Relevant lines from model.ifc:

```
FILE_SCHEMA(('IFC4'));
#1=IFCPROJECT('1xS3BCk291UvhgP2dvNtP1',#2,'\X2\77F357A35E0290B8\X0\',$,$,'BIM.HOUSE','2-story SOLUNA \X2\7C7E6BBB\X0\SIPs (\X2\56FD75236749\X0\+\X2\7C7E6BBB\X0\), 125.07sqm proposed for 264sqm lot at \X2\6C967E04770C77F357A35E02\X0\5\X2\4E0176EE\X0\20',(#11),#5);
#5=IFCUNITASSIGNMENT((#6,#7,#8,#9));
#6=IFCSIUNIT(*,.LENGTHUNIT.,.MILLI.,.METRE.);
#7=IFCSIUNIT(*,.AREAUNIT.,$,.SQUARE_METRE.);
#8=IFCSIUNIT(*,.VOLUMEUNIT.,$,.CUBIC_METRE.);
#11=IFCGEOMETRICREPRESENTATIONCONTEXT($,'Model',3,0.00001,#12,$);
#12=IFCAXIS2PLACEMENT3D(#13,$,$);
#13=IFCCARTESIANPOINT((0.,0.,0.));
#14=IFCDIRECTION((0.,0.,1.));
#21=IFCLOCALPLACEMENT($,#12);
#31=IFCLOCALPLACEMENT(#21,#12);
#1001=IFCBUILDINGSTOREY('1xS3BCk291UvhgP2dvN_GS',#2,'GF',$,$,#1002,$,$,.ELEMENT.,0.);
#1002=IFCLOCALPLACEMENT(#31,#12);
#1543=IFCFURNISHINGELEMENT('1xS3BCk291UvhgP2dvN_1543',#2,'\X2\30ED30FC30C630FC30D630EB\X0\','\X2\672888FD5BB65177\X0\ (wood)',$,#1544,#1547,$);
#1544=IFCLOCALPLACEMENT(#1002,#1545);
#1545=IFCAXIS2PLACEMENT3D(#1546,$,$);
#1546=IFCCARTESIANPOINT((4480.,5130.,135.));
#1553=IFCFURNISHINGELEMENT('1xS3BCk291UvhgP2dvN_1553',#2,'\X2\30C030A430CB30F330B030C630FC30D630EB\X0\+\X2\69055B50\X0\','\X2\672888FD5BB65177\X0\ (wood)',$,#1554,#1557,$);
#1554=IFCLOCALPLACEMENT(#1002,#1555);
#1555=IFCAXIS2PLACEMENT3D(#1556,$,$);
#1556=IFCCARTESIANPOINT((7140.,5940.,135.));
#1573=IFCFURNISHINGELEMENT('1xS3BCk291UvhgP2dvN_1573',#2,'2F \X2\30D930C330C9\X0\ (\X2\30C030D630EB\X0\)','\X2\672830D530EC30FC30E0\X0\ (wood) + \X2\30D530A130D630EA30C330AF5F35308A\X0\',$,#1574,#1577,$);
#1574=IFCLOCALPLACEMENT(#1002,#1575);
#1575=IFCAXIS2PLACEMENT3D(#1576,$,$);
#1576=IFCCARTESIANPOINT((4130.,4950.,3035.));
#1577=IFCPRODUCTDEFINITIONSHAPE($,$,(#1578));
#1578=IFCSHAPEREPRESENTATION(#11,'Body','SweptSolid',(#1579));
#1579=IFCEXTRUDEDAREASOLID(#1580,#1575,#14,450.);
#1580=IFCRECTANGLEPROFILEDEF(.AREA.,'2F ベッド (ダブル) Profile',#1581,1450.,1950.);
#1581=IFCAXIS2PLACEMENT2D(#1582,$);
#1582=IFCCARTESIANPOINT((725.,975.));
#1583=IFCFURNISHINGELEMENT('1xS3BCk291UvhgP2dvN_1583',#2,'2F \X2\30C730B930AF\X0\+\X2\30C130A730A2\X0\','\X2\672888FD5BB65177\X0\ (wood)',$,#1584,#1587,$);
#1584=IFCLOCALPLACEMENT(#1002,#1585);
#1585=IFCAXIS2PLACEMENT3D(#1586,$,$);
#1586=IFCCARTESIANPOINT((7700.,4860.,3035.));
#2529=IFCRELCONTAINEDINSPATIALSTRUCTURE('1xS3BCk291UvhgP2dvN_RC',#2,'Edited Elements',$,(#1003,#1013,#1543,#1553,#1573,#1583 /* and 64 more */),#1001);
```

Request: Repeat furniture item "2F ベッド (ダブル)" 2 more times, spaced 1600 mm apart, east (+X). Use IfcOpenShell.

```python
import numpy as np
import ifcopenshell
import ifcopenshell.api.geometry
import ifcopenshell.api.root
import ifcopenshell.util.element
import ifcopenshell.util.placement
import ifcopenshell.util.unit

model = ifcopenshell.open("model.ifc")
unit_scale = ifcopenshell.util.unit.calculate_unit_scale(model)


def reuse_history(source, copy):
    """copy_class also copies each property set's owner history, people and application; keep the originals."""
    for rel in copy.IsDefinedBy:
        if rel.is_a("IfcRelDefinesByProperties") and (history := rel.RelatingPropertyDefinition.OwnerHistory):
            rel.RelatingPropertyDefinition.OwnerHistory = source.OwnerHistory
            ifcopenshell.util.element.remove_deep2(model, history)


source = model.by_guid("1xS3BCk291UvhgP2dvN_1573")
base = ifcopenshell.util.placement.get_local_placement(source.ObjectPlacement)
step = np.array([1.0, 0.0, 0.0]) * 1.6 / unit_scale

for i in range(1, 3):
    copy = ifcopenshell.api.root.copy_class(model, product=source)
    copy.Representation = ifcopenshell.util.element.copy_deep(
        model, source.Representation, exclude=["IfcGeometricRepresentationContext", "IfcRepresentationMap"]
    )
    reuse_history(source, copy)
    matrix = base.copy()
    matrix[:3, 3] += i * step
    print("added at", matrix[:3, 3].round(3) + 0.0)
    ifcopenshell.api.geometry.edit_object_placement(model, product=copy, matrix=matrix, is_si=False)

model.write("model_rev.ifc")
```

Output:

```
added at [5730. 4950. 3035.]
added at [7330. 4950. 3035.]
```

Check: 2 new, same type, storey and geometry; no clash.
